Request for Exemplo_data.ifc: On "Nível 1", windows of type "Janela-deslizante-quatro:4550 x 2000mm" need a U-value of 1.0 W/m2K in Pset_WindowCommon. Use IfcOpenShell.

First a look at what the model holds.

```python
import ifcopenshell
import ifcopenshell.util.element

model = ifcopenshell.open("Exemplo_data.ifc")
print(model.schema)
storey = next(s for s in model.by_type("IfcBuildingStorey") if s.Name == "Nível 1")
windows = [e for e in ifcopenshell.util.element.get_decomposition(storey) if e.is_a("IfcWindow")]
seen = {}
for e in windows:
    element_type = ifcopenshell.util.element.get_type(e)
    key = (element_type.Name if element_type != e and element_type else None, ifcopenshell.util.element.get_pset(e, "Pset_WindowCommon", "ThermalTransmittance"))
    seen[key] = seen.get(key, 0) + 1
for (name, value), count in sorted(seen.items(), key=str):
    print(count, "x", name, "|", value)
```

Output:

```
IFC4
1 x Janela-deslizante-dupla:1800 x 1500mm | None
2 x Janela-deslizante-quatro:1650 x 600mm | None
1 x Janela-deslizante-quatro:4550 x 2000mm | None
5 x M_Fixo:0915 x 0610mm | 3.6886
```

```python
import ifcopenshell
import ifcopenshell.api.pset
import ifcopenshell.util.element

model = ifcopenshell.open("Exemplo_data.ifc")

storey = next(s for s in model.by_type("IfcBuildingStorey") if s.Name == "Nível 1")
windows = [e for e in ifcopenshell.util.element.get_decomposition(storey) if e.is_a("IfcWindow")]

count = 0
for e in windows:
    element_type = ifcopenshell.util.element.get_type(e)
    if element_type in (None, e) or element_type.Name != "Janela-deslizante-quatro:4550 x 2000mm":
        continue
    # add_pset returns the element's existing set when there is one.
    pset = ifcopenshell.api.pset.add_pset(model, product=e, name="Pset_WindowCommon")
    ifcopenshell.api.pset.edit_pset(model, pset=pset, properties={"ThermalTransmittance": 1.0})
    count += 1

print(count, "windows updated")

model.write("Exemplo_data_v2.ifc")
```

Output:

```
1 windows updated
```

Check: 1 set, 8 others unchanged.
